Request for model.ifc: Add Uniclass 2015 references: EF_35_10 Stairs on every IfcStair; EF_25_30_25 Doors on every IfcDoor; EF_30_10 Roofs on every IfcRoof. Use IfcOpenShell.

First a look at what the model holds.

```python
import ifcopenshell

model = ifcopenshell.open("model.ifc")
print(model.schema)
print("classifications:", [c.Name for c in model.by_type("IfcClassification")])
for ifc_class in ("IfcDoor", "IfcRoof", "IfcStair", "IfcWall", "IfcWindow"):
    print(ifc_class, len(model.by_type(ifc_class)))
```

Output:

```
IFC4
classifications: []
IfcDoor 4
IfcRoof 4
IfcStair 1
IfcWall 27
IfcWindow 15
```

```python
import ifcopenshell
import ifcopenshell.api.classification

model = ifcopenshell.open("model.ifc")

system = ifcopenshell.api.classification.add_classification(model, classification="Uniclass 2015")

codes = {
    "IfcStair": ("EF_35_10", "Stairs"),
    "IfcDoor": ("EF_25_30_25", "Doors"),
    "IfcRoof": ("EF_30_10", "Roofs"),
}
for ifc_class, (code, name) in codes.items():
    products = model.by_type(ifc_class)
    ifcopenshell.api.classification.add_reference(
        model, products=products, classification=system, identification=code, name=name
    )
    print(code, len(products))

model.write("model_updated.ifc")
```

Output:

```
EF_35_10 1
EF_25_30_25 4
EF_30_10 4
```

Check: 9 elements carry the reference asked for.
